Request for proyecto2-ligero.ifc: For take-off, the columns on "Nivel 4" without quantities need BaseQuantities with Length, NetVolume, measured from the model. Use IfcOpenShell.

First a look at what the model holds.

```python
import ifcopenshell
import ifcopenshell.util.element
import ifcopenshell.util.unit

model = ifcopenshell.open("proyecto2-ligero.ifc")
print(model.schema)
for unit_type in ("LENGTHUNIT", "AREAUNIT", "VOLUMEUNIT"):
    print(unit_type, ifcopenshell.util.unit.calculate_unit_scale(model, unit_type))
storey = next(s for s in model.by_type("IfcBuildingStorey") if s.Name == "Nivel 4")
columns = [e for e in ifcopenshell.util.element.get_decomposition(storey) if e.is_a("IfcColumn")]
for e in sorted(columns, key=lambda e: e.id()):
    print(e.id(), e.is_a(), e.Name, list(ifcopenshell.util.element.get_psets(e, qtos_only=True)), sep=" | ")
```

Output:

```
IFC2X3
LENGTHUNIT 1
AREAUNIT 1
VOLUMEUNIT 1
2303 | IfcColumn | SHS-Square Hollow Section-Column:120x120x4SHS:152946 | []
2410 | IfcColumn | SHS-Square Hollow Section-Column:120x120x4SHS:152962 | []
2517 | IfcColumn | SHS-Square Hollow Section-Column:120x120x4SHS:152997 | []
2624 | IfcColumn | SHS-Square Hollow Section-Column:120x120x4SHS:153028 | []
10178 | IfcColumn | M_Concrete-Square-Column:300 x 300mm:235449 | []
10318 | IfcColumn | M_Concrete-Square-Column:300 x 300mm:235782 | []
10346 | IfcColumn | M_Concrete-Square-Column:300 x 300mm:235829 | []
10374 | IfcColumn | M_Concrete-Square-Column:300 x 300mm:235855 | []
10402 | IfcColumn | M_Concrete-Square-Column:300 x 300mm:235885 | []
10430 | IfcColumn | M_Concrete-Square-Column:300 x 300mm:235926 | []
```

```python
import ifcopenshell
import ifcopenshell.api.pset
import ifcopenshell.geom
import ifcopenshell.util.element
import ifcopenshell.util.shape
import ifcopenshell.util.unit

model = ifcopenshell.open("proyecto2-ligero.ifc")
unit_scale = ifcopenshell.util.unit.calculate_unit_scale(model)
volume_scale = ifcopenshell.util.unit.calculate_unit_scale(model, "VOLUMEUNIT")
settings = ifcopenshell.geom.settings()

storey = next(s for s in model.by_type("IfcBuildingStorey") if s.Name == "Nivel 4")
columns = [e for e in ifcopenshell.util.element.get_decomposition(storey) if e.is_a("IfcColumn")]

for e in sorted(columns, key=lambda e: e.id()):
    if ifcopenshell.util.element.get_psets(e, qtos_only=True, should_inherit=False):
        continue
    # Geometry comes back in metres, in the element's own axes.
    shape = ifcopenshell.geom.create_shape(settings, e)
    values = {
        "Length": ifcopenshell.util.shape.get_z(shape.geometry) / unit_scale,
        "NetVolume": ifcopenshell.util.shape.get_volume(shape.geometry) / volume_scale,
    }
    qto = ifcopenshell.api.pset.add_qto(model, product=e, name="BaseQuantities")
    ifcopenshell.api.pset.edit_qto(model, qto=qto, properties=values)
    print(e.id(), {k: round(v, 3) for k, v in values.items()})

model.write("proyecto2-ligero_v2.ifc")
```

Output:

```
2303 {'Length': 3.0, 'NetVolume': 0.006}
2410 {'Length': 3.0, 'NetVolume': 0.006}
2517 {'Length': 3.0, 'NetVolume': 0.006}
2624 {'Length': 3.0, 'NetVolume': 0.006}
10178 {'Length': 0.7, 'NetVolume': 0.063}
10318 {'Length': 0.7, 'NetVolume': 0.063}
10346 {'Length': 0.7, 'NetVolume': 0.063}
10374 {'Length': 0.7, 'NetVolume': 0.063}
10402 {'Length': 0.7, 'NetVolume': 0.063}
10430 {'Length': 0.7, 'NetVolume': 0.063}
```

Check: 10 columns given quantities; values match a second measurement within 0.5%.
